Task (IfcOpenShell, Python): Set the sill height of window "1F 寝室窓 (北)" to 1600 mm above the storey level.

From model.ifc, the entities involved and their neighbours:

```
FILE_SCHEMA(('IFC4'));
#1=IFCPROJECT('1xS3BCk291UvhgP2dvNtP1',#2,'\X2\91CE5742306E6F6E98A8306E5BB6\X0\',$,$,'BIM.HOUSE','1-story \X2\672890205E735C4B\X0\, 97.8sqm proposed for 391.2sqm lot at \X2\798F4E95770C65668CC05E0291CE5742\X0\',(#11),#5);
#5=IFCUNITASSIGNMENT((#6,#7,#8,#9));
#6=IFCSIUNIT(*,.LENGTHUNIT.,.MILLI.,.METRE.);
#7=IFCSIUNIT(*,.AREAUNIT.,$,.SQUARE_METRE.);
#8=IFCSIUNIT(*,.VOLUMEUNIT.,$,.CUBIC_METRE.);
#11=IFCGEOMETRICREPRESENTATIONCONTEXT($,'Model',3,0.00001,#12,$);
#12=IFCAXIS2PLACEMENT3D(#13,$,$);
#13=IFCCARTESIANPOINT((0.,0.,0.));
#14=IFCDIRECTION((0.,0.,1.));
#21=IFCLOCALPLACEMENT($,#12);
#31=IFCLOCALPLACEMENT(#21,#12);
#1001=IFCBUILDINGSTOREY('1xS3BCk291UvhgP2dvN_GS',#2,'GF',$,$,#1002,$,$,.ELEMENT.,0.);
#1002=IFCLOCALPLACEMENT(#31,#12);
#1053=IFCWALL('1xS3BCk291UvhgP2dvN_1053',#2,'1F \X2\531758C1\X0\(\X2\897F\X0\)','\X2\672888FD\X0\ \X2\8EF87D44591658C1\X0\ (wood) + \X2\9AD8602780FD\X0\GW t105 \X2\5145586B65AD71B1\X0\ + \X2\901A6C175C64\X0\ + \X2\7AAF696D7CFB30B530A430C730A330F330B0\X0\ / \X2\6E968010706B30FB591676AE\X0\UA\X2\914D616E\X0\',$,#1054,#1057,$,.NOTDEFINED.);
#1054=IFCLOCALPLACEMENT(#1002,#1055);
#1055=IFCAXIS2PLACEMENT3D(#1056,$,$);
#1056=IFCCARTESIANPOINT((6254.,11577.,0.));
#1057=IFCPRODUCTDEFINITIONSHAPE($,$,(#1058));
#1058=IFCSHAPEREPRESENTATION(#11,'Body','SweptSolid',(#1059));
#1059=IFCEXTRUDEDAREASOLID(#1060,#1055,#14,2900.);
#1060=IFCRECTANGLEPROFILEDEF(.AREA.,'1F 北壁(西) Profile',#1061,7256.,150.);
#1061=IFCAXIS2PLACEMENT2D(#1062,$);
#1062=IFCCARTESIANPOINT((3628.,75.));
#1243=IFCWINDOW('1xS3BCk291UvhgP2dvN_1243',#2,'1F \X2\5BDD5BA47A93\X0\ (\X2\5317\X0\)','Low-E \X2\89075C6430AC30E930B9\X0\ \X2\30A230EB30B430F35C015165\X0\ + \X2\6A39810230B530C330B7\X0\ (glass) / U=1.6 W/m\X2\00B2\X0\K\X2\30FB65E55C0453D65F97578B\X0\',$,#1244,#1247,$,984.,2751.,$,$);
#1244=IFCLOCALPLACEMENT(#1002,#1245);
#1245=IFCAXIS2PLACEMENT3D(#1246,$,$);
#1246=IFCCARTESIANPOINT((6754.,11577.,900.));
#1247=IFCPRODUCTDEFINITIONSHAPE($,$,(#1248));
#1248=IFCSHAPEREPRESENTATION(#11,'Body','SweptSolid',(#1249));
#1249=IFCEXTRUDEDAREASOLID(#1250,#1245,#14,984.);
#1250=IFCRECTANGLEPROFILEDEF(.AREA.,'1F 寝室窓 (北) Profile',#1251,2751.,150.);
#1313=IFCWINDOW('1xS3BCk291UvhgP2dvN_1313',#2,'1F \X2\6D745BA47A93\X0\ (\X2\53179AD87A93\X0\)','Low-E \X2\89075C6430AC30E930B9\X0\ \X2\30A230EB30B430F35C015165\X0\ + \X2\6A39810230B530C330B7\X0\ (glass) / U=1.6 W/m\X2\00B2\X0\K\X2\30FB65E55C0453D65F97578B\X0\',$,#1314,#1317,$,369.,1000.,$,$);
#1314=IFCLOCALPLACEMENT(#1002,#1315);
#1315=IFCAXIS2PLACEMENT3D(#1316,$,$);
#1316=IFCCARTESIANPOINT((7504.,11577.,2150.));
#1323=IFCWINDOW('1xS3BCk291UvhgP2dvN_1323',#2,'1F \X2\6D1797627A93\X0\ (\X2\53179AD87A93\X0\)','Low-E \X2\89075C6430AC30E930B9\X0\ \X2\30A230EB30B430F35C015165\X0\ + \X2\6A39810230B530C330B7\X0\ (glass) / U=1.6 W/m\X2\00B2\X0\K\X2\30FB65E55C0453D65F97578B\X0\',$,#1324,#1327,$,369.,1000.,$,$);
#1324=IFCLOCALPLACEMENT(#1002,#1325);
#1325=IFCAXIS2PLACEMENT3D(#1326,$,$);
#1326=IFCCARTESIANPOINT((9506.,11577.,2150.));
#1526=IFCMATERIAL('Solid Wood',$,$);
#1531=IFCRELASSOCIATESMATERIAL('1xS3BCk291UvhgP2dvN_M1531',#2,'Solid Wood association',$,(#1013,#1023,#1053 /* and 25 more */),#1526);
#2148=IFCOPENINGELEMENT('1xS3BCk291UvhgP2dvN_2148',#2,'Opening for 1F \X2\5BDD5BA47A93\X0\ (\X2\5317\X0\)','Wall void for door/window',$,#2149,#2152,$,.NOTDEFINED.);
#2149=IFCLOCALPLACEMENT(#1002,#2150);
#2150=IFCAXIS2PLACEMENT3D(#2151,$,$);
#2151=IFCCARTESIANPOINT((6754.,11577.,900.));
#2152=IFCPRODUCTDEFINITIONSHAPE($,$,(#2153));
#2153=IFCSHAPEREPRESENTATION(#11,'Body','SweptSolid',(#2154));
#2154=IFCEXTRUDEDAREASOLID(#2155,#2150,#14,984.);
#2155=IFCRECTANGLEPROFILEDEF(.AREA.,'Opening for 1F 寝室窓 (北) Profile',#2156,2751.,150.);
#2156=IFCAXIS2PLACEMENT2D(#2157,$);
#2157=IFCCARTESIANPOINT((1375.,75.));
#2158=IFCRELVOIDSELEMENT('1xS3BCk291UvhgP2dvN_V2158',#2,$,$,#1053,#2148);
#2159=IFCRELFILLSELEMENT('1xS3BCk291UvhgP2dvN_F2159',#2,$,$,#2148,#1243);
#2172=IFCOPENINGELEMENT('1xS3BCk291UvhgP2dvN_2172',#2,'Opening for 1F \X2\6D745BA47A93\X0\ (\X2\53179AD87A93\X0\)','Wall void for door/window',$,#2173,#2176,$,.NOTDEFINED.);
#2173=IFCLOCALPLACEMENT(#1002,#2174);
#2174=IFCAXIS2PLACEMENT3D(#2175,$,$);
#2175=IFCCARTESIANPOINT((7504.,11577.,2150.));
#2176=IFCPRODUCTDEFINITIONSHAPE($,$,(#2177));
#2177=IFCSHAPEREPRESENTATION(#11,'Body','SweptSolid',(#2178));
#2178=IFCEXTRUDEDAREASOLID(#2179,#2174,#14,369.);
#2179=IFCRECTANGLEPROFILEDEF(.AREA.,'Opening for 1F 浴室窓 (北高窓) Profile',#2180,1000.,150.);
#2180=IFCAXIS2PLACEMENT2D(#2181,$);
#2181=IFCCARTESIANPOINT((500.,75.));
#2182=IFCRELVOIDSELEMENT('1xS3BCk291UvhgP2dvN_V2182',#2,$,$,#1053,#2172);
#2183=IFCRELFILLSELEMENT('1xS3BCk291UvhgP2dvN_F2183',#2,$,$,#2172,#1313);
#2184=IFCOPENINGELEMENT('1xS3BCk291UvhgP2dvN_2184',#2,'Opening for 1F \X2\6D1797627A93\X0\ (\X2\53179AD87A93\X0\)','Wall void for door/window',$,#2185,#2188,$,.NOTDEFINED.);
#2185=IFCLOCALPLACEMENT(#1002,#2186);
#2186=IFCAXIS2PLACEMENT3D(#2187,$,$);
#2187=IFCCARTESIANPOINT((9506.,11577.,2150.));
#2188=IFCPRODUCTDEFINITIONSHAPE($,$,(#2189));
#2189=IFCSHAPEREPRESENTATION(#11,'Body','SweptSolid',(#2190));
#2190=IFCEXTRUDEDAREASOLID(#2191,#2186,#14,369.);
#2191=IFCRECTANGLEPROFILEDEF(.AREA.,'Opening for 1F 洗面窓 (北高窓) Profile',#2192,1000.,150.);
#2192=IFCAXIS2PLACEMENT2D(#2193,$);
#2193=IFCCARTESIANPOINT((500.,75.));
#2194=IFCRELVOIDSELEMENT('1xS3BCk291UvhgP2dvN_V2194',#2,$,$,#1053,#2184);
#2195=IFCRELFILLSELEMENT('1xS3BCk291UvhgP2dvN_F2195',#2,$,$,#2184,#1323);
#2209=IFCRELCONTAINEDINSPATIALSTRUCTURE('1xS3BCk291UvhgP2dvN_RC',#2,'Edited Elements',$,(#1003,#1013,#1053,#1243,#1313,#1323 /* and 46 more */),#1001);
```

```python
import numpy as np
import ifcopenshell
import ifcopenshell.api.geometry
import ifcopenshell.geom
import ifcopenshell.util.element
import ifcopenshell.util.placement
import ifcopenshell.util.shape
import ifcopenshell.util.unit

model = ifcopenshell.open("model.ifc")
unit_scale = ifcopenshell.util.unit.calculate_unit_scale(model)

window = model.by_guid("1xS3BCk291UvhgP2dvN_1243")
opening = window.FillsVoids[0].RelatingOpeningElement
storey = ifcopenshell.util.element.get_container(window, ifc_class="IfcBuildingStorey")
level = ifcopenshell.util.placement.get_local_placement(storey.ObjectPlacement)[2, 3]

# The opening's origin need not be at the sill, so measure its lowest point.
shape = ifcopenshell.geom.create_shape(ifcopenshell.geom.settings(), opening)
bottom = ifcopenshell.util.shape.get_shape_bottom_elevation(shape, shape.geometry) / unit_scale
dz = level + 1600.0 - bottom

shift = np.array([0.0, 0.0, dz])
# The window is not placed relative to its opening, so move both.
for product in (opening, window):
    matrix = ifcopenshell.util.placement.get_local_placement(product.ObjectPlacement)
    matrix[:3, 3] += shift
    ifcopenshell.api.geometry.edit_object_placement(model, product=product, matrix=matrix, is_si=False)

print(f"moved by {dz * unit_scale:+.3f} m")

model.write("model_updated.ifc")
```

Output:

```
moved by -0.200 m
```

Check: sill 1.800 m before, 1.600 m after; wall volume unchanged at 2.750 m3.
